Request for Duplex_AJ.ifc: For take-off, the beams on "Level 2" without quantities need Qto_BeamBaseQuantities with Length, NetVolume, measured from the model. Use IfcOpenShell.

First a look at what the model holds.

```python
import ifcopenshell
import ifcopenshell.util.element
import ifcopenshell.util.unit

model = ifcopenshell.open("Duplex_AJ.ifc")
print(model.schema)
for unit_type in ("LENGTHUNIT", "AREAUNIT", "VOLUMEUNIT"):
    print(unit_type, ifcopenshell.util.unit.calculate_unit_scale(model, unit_type))
storey = next(s for s in model.by_type("IfcBuildingStorey") if s.Name == "Level 2")
beams = [e for e in ifcopenshell.util.element.get_decomposition(storey) if e.is_a("IfcBeam")]
for e in sorted(beams, key=lambda e: e.id()):
    print(e.id(), e.is_a(), e.Name, list(ifcopenshell.util.element.get_psets(e, qtos_only=True)), sep=" | ")
```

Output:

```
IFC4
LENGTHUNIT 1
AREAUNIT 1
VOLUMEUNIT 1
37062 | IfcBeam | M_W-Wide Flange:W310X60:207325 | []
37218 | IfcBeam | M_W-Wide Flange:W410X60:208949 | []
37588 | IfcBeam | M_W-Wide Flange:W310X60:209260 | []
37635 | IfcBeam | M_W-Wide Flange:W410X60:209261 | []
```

```python
import ifcopenshell
import ifcopenshell.api.pset
import ifcopenshell.geom
import ifcopenshell.util.element
import ifcopenshell.util.shape
import ifcopenshell.util.unit

model = ifcopenshell.open("Duplex_AJ.ifc")
unit_scale = ifcopenshell.util.unit.calculate_unit_scale(model)
volume_scale = ifcopenshell.util.unit.calculate_unit_scale(model, "VOLUMEUNIT")
settings = ifcopenshell.geom.settings()

storey = next(s for s in model.by_type("IfcBuildingStorey") if s.Name == "Level 2")
beams = [e for e in ifcopenshell.util.element.get_decomposition(storey) if e.is_a("IfcBeam")]

for e in sorted(beams, key=lambda e: e.id()):
    if ifcopenshell.util.element.get_psets(e, qtos_only=True, should_inherit=False):
        continue
    # Geometry comes back in metres, in the element's own axes.
    shape = ifcopenshell.geom.create_shape(settings, e)
    values = {
        "Length": ifcopenshell.util.shape.get_max_xyz(shape.geometry) / unit_scale,
        "NetVolume": ifcopenshell.util.shape.get_volume(shape.geometry) / volume_scale,
    }
    qto = ifcopenshell.api.pset.add_qto(model, product=e, name="Qto_BeamBaseQuantities")
    ifcopenshell.api.pset.edit_qto(model, qto=qto, properties=values)
    print(e.id(), {k: round(v, 3) for k, v in values.items()})

model.write("Duplex_AJ_v2.ifc")
```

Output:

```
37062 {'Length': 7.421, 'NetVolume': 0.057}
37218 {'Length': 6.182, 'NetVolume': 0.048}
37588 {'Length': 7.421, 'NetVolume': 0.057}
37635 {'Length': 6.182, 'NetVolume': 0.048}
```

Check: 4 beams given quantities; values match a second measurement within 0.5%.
